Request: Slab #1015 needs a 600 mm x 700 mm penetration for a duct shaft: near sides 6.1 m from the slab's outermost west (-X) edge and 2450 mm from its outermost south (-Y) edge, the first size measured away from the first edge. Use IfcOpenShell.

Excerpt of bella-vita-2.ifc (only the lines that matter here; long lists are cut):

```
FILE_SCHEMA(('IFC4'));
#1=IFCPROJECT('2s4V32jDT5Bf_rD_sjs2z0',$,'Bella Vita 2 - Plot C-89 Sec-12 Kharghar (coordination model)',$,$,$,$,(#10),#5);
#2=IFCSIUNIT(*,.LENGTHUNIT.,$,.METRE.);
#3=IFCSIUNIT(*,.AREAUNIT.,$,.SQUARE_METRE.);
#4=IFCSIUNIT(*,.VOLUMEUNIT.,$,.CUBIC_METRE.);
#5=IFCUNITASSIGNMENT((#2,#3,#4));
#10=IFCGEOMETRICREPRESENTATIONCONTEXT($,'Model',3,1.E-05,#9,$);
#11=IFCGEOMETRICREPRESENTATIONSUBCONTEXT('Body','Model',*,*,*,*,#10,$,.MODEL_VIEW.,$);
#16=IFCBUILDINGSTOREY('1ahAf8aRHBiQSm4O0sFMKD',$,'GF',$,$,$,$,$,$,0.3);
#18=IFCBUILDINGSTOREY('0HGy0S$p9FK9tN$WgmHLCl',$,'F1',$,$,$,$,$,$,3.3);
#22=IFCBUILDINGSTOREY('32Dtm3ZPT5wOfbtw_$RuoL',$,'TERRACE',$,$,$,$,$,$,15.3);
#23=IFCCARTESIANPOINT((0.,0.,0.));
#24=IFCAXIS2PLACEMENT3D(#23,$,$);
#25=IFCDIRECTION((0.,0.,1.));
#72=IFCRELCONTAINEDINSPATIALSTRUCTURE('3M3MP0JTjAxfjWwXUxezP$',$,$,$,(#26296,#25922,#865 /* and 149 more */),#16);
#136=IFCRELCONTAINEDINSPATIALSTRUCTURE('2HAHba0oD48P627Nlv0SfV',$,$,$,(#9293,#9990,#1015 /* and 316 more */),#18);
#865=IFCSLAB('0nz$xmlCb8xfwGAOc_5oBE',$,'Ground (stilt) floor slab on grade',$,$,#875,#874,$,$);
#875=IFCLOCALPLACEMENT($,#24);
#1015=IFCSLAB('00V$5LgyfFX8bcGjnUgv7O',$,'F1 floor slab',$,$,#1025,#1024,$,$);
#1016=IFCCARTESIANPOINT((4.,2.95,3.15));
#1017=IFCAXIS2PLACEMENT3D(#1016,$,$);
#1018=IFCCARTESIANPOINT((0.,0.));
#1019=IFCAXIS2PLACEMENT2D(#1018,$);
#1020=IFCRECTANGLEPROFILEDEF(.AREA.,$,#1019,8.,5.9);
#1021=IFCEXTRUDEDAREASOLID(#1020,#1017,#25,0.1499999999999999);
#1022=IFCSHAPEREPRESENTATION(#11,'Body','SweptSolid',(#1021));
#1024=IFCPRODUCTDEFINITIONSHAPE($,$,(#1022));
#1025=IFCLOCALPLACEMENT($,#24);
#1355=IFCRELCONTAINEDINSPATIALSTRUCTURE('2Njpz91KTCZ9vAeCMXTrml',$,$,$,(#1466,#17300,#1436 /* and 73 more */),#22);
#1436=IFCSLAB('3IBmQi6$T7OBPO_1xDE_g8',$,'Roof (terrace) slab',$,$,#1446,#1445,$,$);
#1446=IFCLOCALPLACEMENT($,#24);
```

```python
import numpy as np
import ifcopenshell
import ifcopenshell.api.feature
import ifcopenshell.api.geometry
import ifcopenshell.api.root
import ifcopenshell.geom
import ifcopenshell.util.placement
import ifcopenshell.util.representation
import ifcopenshell.util.shape
import ifcopenshell.util.unit

model = ifcopenshell.open("bella-vita-2.ifc")
unit_scale = ifcopenshell.util.unit.calculate_unit_scale(model)
settings = ifcopenshell.geom.settings()


def volume(element):
    """Net volume in cubic metres, openings subtracted."""
    shape = ifcopenshell.geom.create_shape(settings, element)
    return ifcopenshell.util.shape.get_volume(shape.geometry)


slab = model.by_id(1015)
before = volume(slab)

# Extent in the slab's own axes, in metres. The edges named are its -X and -Y sides.
slab_shape = ifcopenshell.geom.create_shape(settings, slab)
vertices = ifcopenshell.util.shape.get_vertices(slab_shape.geometry)
x_min, y_min, bottom = vertices.min(axis=0)
top = vertices[:, 2].max()

opening = ifcopenshell.api.root.create_entity(model, ifc_class="IfcOpeningElement", name="Duct shaft opening", predefined_type="OPENING")
context = ifcopenshell.util.representation.get_context(model, "Model", "Body", "MODEL_VIEW")
width, depth = 0.6, 0.7
outline = [(0.0, 0.0), (width, 0.0), (width, depth), (0.0, depth), (0.0, 0.0)]
# Overshoot both faces by 50 mm so the cut is clean.
shape = ifcopenshell.api.geometry.add_slab_representation(
    model, context=context, depth=top - bottom + 0.1, polyline=outline
)
ifcopenshell.api.geometry.assign_representation(model, product=opening, representation=shape)

matrix = ifcopenshell.util.placement.get_local_placement(slab.ObjectPlacement)
matrix[:, 3] = matrix @ np.append(np.array([x_min + 6.1, y_min + 2.45, bottom - 0.05]) / unit_scale, 1.0)
ifcopenshell.api.geometry.edit_object_placement(model, product=opening, matrix=matrix, is_si=False)
ifcopenshell.api.feature.add_feature(model, feature=opening, element=slab)

after = volume(slab)

print(f"slab volume {before:.3f} -> {after:.3f} m3")

model.write("bella-vita-2_edited.ifc")
```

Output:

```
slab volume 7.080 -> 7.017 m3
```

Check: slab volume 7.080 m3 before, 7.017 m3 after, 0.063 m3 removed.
